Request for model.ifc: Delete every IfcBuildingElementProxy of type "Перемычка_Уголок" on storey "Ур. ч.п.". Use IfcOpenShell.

First a look at what the model holds.

```python
import ifcopenshell
import ifcopenshell.util.element

model = ifcopenshell.open("model.ifc")
print(model.schema)
storey = next(s for s in model.by_type("IfcBuildingStorey") if s.Name == "Ур. ч.п.")
proxies = [e for e in ifcopenshell.util.element.get_decomposition(storey) if e.is_a("IfcBuildingElementProxy")]
seen = {}
for e in proxies:
    element_type = ifcopenshell.util.element.get_type(e)
    name = element_type.Name if element_type not in (None, e) else None
    seen[name] = seen.get(name, 0) + 1
for name, count in sorted(seen.items(), key=str):
    print(count, "x", name)
```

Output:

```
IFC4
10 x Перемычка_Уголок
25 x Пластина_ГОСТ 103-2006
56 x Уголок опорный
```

```python
import ifcopenshell
import ifcopenshell.api.root
import ifcopenshell.util.element

model = ifcopenshell.open("model.ifc")

storey = next(s for s in model.by_type("IfcBuildingStorey") if s.Name == "Ур. ч.п.")
proxies = [e for e in ifcopenshell.util.element.get_decomposition(storey) if e.is_a("IfcBuildingElementProxy")]
targets = [e for e in proxies if (t := ifcopenshell.util.element.get_type(e)) not in (None, e) and t.Name == "Перемычка_Уголок"]

for e in targets:
    ifcopenshell.api.root.remove_product(model, product=e)
print(len(targets), "removed")

model.write("model_edited.ifc")
```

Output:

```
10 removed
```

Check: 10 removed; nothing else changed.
